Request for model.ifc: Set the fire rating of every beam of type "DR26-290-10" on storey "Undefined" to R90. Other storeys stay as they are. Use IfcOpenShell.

First a look at what the model holds.

```python
import ifcopenshell
import ifcopenshell.util.element

model = ifcopenshell.open("model.ifc")
print(model.schema)
storey = next(s for s in model.by_type("IfcBuildingStorey") if s.Name == "Undefined")
beams = [e for e in ifcopenshell.util.element.get_decomposition(storey) if e.is_a("IfcBeam")]
seen = {}
for e in beams:
    element_type = ifcopenshell.util.element.get_type(e)
    key = (element_type.Name if element_type != e and element_type else None, ifcopenshell.util.element.get_pset(e, "Pset_BeamCommon", "FireRating"))
    seen[key] = seen.get(key, 0) + 1
for (name, value), count in sorted(seen.items(), key=str):
    print(count, "x", name, "|", value)
```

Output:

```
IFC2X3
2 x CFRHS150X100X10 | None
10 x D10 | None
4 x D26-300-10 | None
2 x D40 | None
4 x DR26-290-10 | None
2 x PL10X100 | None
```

```python
import ifcopenshell
import ifcopenshell.api.pset
import ifcopenshell.util.element

model = ifcopenshell.open("model.ifc")

storey = next(s for s in model.by_type("IfcBuildingStorey") if s.Name == "Undefined")
beams = [e for e in ifcopenshell.util.element.get_decomposition(storey) if e.is_a("IfcBeam")]

count = 0
for e in beams:
    element_type = ifcopenshell.util.element.get_type(e)
    if element_type in (None, e) or element_type.Name != "DR26-290-10":
        continue
    found = ifcopenshell.util.element.get_pset(e, "Pset_BeamCommon", should_inherit=False)
    if found:
        pset = model.by_id(found["id"])
        if len(ifcopenshell.util.element.get_elements_by_pset(pset)) > 1:
            pset = ifcopenshell.api.pset.unshare_pset(model, products=[e], pset=pset)[0]
    else:
        pset = ifcopenshell.api.pset.add_pset(model, product=e, name="Pset_BeamCommon")
    ifcopenshell.api.pset.edit_pset(model, pset=pset, properties={"FireRating": "R90"})
    count += 1

print(count, "beams updated")

model.write("model_edited.ifc")
```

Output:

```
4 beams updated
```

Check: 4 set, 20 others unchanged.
